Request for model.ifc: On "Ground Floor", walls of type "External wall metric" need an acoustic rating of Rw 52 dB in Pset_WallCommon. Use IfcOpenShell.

First a look at what the model holds.

```python
import ifcopenshell
import ifcopenshell.util.element

model = ifcopenshell.open("model.ifc")
print(model.schema)
storey = next(s for s in model.by_type("IfcBuildingStorey") if s.Name == "Ground Floor")
walls = [e for e in ifcopenshell.util.element.get_decomposition(storey) if e.is_a("IfcWall")]
seen = {}
for e in walls:
    element_type = ifcopenshell.util.element.get_type(e)
    key = (element_type.Name if element_type != e and element_type else None, ifcopenshell.util.element.get_pset(e, "Pset_WallCommon", "AcousticRating"))
    seen[key] = seen.get(key, 0) + 1
for (name, value), count in sorted(seen.items(), key=str):
    print(count, "x", name, "|", value)
```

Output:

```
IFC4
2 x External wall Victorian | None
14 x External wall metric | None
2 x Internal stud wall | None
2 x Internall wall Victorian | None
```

```python
import ifcopenshell
import ifcopenshell.api.pset
import ifcopenshell.util.element

model = ifcopenshell.open("model.ifc")

storey = next(s for s in model.by_type("IfcBuildingStorey") if s.Name == "Ground Floor")
walls = [e for e in ifcopenshell.util.element.get_decomposition(storey) if e.is_a("IfcWall")]

count = 0
for e in walls:
    element_type = ifcopenshell.util.element.get_type(e)
    if element_type in (None, e) or element_type.Name != "External wall metric":
        continue
    # add_pset returns the element's existing set when there is one.
    pset = ifcopenshell.api.pset.add_pset(model, product=e, name="Pset_WallCommon")
    ifcopenshell.api.pset.edit_pset(model, pset=pset, properties={"AcousticRating": "Rw 52 dB"})
    count += 1

print(count, "walls updated")

model.write("model_v2.ifc")
```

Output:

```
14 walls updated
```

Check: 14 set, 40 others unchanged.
